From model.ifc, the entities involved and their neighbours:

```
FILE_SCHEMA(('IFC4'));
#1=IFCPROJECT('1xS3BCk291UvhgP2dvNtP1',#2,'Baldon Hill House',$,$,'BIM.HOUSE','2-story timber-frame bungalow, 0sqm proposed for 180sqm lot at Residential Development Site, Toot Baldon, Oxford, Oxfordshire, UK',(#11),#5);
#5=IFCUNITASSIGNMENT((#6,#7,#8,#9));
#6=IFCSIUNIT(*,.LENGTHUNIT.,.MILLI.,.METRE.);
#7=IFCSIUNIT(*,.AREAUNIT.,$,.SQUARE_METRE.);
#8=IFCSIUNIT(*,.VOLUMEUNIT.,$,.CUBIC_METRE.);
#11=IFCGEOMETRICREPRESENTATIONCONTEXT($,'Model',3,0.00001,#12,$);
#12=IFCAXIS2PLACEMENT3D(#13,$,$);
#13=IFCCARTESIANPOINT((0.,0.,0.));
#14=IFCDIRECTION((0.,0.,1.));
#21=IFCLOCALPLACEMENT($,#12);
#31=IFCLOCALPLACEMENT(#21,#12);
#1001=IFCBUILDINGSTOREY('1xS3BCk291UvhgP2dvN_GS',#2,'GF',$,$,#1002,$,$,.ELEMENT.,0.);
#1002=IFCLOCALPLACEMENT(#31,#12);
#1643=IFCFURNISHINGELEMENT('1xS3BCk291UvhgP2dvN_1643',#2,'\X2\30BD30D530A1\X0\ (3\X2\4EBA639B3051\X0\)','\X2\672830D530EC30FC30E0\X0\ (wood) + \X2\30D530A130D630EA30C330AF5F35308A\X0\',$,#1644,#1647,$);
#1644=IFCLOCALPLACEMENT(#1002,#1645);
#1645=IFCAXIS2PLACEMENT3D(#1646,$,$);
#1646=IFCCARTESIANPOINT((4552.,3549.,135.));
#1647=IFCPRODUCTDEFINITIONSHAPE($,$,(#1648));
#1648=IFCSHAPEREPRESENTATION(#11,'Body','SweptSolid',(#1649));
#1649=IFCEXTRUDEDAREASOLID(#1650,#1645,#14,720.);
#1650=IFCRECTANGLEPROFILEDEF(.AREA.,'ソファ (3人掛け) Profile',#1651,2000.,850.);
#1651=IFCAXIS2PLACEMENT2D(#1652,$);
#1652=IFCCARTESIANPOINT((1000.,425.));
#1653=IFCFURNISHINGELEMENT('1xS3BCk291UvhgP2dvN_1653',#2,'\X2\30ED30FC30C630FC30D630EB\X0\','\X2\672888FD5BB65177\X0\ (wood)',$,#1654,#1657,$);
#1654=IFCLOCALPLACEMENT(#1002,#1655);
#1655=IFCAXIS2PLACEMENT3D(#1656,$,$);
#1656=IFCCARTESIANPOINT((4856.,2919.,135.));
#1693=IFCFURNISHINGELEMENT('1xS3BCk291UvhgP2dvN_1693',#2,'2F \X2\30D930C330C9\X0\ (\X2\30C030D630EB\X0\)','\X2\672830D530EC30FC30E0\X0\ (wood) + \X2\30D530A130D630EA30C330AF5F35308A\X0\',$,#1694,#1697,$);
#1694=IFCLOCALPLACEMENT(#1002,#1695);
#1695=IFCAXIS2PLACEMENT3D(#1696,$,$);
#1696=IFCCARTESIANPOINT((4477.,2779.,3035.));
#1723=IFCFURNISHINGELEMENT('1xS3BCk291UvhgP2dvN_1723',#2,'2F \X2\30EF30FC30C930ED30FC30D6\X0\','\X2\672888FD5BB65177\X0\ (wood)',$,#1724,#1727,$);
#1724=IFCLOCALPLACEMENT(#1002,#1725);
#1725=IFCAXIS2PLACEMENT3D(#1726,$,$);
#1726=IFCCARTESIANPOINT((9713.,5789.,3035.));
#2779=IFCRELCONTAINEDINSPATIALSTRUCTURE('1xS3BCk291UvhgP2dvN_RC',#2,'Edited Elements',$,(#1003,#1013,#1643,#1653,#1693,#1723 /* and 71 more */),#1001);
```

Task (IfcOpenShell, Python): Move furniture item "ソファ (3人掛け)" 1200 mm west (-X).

```python
import ifcopenshell
import ifcopenshell.api.geometry
import ifcopenshell.util.placement
import ifcopenshell.util.unit

model = ifcopenshell.open("model.ifc")
unit_scale = ifcopenshell.util.unit.calculate_unit_scale(model)

item = model.by_guid("1xS3BCk291UvhgP2dvN_1643")
matrix = ifcopenshell.util.placement.get_local_placement(item.ObjectPlacement)
matrix[0, 3] -= 1.2 / unit_scale
ifcopenshell.api.geometry.edit_object_placement(model, product=item, matrix=matrix, is_si=False)

print(ifcopenshell.util.placement.get_local_placement(item.ObjectPlacement).round(3) + 0.0)

model.write("model_updated.ifc")
```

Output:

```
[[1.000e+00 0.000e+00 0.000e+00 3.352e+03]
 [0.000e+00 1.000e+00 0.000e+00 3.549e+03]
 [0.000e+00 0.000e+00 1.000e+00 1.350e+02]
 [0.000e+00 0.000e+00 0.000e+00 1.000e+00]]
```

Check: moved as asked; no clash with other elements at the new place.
